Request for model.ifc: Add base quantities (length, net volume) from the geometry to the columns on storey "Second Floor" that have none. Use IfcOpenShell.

First a look at what the model holds.

```python
import ifcopenshell
import ifcopenshell.util.element
import ifcopenshell.util.unit

model = ifcopenshell.open("model.ifc")
print(model.schema)
for unit_type in ("LENGTHUNIT", "AREAUNIT", "VOLUMEUNIT"):
    print(unit_type, ifcopenshell.util.unit.calculate_unit_scale(model, unit_type))
storey = next(s for s in model.by_type("IfcBuildingStorey") if s.Name == "Second Floor")
columns = [e for e in ifcopenshell.util.element.get_decomposition(storey) if e.is_a("IfcColumn")]
for e in sorted(columns, key=lambda e: e.id()):
    print(e.id(), e.is_a(), e.Name, list(ifcopenshell.util.element.get_psets(e, qtos_only=True)), sep=" | ")
```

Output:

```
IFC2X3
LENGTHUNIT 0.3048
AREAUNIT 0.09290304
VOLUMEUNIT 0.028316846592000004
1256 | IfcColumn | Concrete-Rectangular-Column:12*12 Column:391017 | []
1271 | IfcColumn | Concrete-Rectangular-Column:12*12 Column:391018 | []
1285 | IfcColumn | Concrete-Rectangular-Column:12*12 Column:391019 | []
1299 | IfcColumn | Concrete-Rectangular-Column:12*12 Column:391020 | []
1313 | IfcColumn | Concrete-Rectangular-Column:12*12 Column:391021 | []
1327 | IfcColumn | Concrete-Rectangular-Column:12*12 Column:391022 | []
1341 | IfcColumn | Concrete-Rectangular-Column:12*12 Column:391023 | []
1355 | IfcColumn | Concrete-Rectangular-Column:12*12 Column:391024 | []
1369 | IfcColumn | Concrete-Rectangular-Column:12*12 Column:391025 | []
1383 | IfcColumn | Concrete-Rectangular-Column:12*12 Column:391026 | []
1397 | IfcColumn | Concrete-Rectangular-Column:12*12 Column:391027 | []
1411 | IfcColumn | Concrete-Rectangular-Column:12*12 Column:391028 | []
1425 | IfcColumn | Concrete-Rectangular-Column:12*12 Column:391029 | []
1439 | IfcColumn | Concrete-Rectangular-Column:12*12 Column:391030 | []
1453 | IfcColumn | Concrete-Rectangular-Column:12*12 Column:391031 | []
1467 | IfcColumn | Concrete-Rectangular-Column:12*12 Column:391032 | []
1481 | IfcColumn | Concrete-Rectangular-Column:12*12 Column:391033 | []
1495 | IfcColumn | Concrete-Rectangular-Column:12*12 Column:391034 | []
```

```python
import ifcopenshell
import ifcopenshell.api.pset
import ifcopenshell.geom
import ifcopenshell.util.element
import ifcopenshell.util.shape
import ifcopenshell.util.unit

model = ifcopenshell.open("model.ifc")
unit_scale = ifcopenshell.util.unit.calculate_unit_scale(model)
volume_scale = ifcopenshell.util.unit.calculate_unit_scale(model, "VOLUMEUNIT")
settings = ifcopenshell.geom.settings()

storey = next(s for s in model.by_type("IfcBuildingStorey") if s.Name == "Second Floor")
columns = [e for e in ifcopenshell.util.element.get_decomposition(storey) if e.is_a("IfcColumn")]

for e in sorted(columns, key=lambda e: e.id()):
    if ifcopenshell.util.element.get_psets(e, qtos_only=True, should_inherit=False):
        continue
    # Geometry comes back in metres, in the element's own axes.
    shape = ifcopenshell.geom.create_shape(settings, e)
    values = {
        "Length": ifcopenshell.util.shape.get_z(shape.geometry) / unit_scale,
        "NetVolume": ifcopenshell.util.shape.get_volume(shape.geometry) / volume_scale,
    }
    qto = ifcopenshell.api.pset.add_qto(model, product=e, name="BaseQuantities")
    ifcopenshell.api.pset.edit_qto(model, qto=qto, properties=values)
    print(e.id(), {k: round(v, 3) for k, v in values.items()})

model.write("model-out.ifc")
```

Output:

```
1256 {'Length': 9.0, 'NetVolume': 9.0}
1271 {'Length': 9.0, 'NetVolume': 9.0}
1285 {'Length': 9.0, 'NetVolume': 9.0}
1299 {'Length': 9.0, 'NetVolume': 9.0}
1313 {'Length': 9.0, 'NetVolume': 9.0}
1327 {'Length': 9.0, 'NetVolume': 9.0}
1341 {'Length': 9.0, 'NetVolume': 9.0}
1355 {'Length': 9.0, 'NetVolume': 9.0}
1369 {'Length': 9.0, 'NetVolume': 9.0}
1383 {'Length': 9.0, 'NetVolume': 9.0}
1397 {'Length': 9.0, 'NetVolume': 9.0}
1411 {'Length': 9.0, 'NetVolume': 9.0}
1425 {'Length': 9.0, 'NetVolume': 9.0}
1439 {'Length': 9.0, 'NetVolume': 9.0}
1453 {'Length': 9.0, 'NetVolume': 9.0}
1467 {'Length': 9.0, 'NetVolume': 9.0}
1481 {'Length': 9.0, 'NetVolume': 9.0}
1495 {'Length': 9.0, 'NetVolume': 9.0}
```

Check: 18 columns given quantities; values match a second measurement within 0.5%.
